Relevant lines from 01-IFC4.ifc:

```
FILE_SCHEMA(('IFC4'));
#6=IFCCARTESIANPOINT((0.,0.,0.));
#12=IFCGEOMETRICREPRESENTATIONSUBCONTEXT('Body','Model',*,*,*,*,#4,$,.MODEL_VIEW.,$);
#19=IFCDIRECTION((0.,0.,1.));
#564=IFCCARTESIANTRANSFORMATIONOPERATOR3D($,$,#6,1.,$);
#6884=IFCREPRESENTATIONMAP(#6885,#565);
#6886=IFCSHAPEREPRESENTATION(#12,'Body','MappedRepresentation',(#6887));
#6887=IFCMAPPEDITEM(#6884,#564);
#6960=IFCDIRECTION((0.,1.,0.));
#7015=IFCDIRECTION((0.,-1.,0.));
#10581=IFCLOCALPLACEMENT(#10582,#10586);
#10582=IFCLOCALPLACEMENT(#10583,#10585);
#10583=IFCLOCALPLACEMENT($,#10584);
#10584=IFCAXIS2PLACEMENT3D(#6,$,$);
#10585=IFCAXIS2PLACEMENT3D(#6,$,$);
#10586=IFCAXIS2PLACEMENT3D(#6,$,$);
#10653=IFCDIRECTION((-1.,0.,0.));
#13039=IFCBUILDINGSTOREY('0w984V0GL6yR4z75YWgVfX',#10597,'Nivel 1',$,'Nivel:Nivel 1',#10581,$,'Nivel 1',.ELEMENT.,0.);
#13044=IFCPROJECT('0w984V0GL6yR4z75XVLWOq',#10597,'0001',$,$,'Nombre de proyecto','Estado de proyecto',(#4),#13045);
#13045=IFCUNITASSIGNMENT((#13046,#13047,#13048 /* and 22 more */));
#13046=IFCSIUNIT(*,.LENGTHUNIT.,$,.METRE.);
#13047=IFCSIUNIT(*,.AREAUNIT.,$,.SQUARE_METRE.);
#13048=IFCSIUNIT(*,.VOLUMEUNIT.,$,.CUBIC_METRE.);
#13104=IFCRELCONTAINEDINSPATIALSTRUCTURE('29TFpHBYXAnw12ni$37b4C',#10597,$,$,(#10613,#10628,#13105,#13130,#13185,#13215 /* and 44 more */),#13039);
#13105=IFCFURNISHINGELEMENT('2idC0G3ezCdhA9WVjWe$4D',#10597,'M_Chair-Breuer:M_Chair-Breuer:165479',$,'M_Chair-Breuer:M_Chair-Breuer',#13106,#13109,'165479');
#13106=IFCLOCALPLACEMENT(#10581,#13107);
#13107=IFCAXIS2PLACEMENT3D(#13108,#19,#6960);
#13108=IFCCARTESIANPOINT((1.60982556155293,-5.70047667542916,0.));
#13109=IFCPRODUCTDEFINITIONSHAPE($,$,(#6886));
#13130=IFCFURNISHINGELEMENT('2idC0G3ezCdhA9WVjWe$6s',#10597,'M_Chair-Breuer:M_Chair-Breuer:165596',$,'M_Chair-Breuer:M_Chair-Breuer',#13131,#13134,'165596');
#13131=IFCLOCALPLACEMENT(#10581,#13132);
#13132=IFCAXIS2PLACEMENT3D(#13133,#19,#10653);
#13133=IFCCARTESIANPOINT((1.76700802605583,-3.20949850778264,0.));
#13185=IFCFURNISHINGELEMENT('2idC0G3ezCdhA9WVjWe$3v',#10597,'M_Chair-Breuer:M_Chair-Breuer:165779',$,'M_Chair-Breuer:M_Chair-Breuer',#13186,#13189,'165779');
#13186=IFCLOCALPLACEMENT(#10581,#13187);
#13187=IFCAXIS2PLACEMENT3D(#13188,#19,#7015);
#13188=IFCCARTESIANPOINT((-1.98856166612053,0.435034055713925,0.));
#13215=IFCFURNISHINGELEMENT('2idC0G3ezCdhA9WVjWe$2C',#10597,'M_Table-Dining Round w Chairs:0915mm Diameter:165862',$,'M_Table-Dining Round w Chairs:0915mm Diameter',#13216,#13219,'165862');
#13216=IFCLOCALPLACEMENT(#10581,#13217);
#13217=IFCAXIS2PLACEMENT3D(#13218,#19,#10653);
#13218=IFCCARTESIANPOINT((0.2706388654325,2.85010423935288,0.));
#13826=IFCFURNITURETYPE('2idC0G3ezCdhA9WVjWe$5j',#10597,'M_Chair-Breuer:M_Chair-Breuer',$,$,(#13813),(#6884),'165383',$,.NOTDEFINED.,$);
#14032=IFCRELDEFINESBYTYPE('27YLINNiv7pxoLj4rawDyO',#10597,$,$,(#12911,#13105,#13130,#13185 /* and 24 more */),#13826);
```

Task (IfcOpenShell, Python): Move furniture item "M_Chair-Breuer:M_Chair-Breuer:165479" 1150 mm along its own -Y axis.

```python
import ifcopenshell
import ifcopenshell.api.geometry
import ifcopenshell.util.placement

model = ifcopenshell.open("01-IFC4.ifc")

item = model.by_id(13105)
matrix = ifcopenshell.util.placement.get_local_placement(item.ObjectPlacement)
matrix[:3, 3] -= matrix[:3, 1] * 1.15
ifcopenshell.api.geometry.edit_object_placement(model, product=item, matrix=matrix, is_si=False)

print(ifcopenshell.util.placement.get_local_placement(item.ObjectPlacement).round(3) + 0.0)

model.write("01-IFC4-out.ifc")
```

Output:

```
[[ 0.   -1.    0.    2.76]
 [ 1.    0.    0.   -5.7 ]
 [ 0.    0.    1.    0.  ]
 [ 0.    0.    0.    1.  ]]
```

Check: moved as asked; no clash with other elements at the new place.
